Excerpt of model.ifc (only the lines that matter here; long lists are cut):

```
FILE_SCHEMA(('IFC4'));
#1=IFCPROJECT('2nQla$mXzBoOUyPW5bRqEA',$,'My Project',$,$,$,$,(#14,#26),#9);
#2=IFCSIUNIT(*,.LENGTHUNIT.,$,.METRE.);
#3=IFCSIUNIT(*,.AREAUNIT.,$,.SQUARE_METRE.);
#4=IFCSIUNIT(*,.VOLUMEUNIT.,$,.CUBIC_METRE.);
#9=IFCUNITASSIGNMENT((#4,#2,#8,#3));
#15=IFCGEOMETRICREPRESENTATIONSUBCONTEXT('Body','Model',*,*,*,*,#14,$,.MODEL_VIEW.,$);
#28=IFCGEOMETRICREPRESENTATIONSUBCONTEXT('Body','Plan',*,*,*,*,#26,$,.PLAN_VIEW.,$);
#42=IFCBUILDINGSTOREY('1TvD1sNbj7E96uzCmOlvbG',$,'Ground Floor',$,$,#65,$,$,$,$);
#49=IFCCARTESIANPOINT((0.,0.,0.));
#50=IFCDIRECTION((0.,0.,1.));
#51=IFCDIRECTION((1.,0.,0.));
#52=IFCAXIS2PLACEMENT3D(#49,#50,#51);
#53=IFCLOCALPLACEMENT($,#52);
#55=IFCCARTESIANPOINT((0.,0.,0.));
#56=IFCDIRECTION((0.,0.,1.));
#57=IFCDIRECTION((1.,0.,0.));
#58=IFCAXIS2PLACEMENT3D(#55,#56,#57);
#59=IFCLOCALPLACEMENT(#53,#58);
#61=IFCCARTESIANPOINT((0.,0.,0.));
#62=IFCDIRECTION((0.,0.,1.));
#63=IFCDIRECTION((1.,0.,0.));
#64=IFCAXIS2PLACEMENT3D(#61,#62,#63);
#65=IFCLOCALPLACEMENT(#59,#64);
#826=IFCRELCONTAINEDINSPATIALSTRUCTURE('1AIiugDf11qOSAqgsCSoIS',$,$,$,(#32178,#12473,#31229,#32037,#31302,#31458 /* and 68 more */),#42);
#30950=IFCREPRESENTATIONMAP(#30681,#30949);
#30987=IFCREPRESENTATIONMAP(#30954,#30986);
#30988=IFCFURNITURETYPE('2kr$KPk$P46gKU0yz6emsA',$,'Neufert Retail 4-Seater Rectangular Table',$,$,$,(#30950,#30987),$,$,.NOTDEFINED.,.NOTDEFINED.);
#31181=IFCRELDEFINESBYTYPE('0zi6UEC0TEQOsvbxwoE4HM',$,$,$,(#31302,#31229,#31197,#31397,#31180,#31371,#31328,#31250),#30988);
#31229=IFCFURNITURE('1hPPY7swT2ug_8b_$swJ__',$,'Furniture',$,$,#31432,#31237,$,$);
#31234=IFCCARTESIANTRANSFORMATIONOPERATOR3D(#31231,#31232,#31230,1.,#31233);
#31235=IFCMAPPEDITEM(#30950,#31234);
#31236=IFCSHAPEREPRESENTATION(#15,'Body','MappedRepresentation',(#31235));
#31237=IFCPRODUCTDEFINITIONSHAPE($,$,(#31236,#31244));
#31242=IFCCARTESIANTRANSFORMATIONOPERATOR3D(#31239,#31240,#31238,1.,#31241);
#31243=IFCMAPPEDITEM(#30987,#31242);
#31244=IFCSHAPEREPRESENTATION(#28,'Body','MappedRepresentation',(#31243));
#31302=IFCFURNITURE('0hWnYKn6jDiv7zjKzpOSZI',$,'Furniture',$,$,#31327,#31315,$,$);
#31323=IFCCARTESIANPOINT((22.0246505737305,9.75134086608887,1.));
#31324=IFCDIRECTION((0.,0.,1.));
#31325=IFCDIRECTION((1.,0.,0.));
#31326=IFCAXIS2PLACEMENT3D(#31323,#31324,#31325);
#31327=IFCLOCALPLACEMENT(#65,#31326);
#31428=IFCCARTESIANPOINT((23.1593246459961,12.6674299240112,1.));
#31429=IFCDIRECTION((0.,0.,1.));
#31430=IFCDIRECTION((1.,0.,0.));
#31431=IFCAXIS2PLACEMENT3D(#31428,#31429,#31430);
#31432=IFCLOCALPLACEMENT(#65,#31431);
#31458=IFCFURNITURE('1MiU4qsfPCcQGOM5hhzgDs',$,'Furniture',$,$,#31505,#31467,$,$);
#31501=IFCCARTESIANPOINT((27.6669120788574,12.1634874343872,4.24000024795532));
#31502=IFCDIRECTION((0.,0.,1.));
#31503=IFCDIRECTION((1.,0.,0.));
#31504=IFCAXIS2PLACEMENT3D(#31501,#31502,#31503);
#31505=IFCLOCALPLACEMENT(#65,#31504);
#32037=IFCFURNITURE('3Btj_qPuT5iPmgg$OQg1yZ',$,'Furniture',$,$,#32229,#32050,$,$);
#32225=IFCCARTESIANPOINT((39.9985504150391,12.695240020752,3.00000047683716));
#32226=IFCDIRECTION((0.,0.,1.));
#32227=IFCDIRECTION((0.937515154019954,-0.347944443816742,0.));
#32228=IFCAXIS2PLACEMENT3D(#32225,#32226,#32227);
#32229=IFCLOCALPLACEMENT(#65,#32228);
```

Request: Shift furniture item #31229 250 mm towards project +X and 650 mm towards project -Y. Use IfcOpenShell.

```python
import ifcopenshell
import ifcopenshell.api.geometry
import ifcopenshell.util.placement
import ifcopenshell.util.unit

model = ifcopenshell.open("model.ifc")
unit_scale = ifcopenshell.util.unit.calculate_unit_scale(model)

item = model.by_id(31229)
matrix = ifcopenshell.util.placement.get_local_placement(item.ObjectPlacement)
matrix[0, 3] += 0.25 / unit_scale
matrix[1, 3] -= 0.65 / unit_scale
ifcopenshell.api.geometry.edit_object_placement(model, product=item, matrix=matrix, is_si=False)

print(ifcopenshell.util.placement.get_local_placement(item.ObjectPlacement).round(3) + 0.0)

model.write("model_rev.ifc")
```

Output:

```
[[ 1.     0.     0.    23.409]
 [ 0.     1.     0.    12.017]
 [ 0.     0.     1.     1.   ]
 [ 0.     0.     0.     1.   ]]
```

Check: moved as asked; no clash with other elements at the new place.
